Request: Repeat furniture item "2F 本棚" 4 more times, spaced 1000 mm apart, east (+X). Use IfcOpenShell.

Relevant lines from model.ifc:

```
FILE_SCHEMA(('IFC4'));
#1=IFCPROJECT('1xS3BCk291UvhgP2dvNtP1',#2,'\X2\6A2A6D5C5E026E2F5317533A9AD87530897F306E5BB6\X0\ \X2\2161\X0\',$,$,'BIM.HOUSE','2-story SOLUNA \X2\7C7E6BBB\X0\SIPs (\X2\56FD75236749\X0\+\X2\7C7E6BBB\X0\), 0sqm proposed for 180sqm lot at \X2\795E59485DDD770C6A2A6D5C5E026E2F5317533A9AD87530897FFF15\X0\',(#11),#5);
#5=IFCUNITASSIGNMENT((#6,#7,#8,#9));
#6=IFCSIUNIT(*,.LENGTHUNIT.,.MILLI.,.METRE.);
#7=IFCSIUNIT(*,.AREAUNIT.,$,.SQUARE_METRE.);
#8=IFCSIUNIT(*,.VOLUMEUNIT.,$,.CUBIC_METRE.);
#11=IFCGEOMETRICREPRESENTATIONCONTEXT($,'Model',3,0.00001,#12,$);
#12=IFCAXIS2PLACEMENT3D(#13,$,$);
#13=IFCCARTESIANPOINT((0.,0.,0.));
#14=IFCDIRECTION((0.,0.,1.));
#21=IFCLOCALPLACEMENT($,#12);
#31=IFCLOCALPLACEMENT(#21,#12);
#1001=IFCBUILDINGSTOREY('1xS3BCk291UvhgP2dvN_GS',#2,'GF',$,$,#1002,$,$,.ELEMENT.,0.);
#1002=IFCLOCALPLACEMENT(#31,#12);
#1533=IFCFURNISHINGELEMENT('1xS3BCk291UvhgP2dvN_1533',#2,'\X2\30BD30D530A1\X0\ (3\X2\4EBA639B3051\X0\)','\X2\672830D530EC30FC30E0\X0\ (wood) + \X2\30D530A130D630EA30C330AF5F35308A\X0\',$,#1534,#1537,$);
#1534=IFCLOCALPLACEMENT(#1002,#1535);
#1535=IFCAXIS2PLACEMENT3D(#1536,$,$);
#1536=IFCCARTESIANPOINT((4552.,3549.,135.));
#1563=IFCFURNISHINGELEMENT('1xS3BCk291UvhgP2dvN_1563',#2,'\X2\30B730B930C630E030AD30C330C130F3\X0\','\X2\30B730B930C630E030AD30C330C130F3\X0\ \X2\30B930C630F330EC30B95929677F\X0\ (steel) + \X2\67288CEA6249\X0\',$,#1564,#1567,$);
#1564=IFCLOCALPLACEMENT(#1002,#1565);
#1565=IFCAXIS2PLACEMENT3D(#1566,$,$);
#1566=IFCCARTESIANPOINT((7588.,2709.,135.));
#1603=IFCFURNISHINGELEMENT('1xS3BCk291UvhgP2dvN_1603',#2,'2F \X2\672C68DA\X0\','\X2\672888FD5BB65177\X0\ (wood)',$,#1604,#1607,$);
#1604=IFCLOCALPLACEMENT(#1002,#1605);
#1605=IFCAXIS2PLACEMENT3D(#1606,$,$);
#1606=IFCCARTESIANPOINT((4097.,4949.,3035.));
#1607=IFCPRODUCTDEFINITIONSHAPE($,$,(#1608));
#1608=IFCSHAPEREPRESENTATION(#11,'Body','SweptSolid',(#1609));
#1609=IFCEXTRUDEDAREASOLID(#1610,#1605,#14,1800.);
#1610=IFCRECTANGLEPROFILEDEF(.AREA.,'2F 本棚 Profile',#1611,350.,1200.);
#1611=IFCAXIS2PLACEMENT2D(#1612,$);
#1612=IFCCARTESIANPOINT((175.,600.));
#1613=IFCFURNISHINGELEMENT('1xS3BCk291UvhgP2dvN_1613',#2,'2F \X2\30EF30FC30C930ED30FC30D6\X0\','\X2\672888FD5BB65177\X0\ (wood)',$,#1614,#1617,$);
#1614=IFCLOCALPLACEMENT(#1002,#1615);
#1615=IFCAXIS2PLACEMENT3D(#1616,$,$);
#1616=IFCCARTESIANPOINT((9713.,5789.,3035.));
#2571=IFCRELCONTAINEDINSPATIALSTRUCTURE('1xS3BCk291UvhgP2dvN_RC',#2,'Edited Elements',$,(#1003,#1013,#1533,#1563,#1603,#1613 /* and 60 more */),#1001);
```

```python
import numpy as np
import ifcopenshell
import ifcopenshell.api.geometry
import ifcopenshell.api.root
import ifcopenshell.util.element
import ifcopenshell.util.placement
import ifcopenshell.util.unit

model = ifcopenshell.open("model.ifc")
unit_scale = ifcopenshell.util.unit.calculate_unit_scale(model)


def reuse_history(source, copy):
    """copy_class also copies each property set's owner history, people and application; keep the originals."""
    for rel in copy.IsDefinedBy:
        if rel.is_a("IfcRelDefinesByProperties") and (history := rel.RelatingPropertyDefinition.OwnerHistory):
            rel.RelatingPropertyDefinition.OwnerHistory = source.OwnerHistory
            ifcopenshell.util.element.remove_deep2(model, history)


source = model.by_guid("1xS3BCk291UvhgP2dvN_1603")
base = ifcopenshell.util.placement.get_local_placement(source.ObjectPlacement)
step = np.array([1.0, 0.0, 0.0]) * 1 / unit_scale

for i in range(1, 5):
    copy = ifcopenshell.api.root.copy_class(model, product=source)
    copy.Representation = ifcopenshell.util.element.copy_deep(
        model, source.Representation, exclude=["IfcGeometricRepresentationContext", "IfcRepresentationMap"]
    )
    reuse_history(source, copy)
    matrix = base.copy()
    matrix[:3, 3] += i * step
    print("added at", matrix[:3, 3].round(3) + 0.0)
    ifcopenshell.api.geometry.edit_object_placement(model, product=copy, matrix=matrix, is_si=False)

model.write("model_v2.ifc")
```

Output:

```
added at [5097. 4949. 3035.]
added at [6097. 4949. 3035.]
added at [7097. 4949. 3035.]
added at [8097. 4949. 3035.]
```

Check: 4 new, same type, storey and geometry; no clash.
